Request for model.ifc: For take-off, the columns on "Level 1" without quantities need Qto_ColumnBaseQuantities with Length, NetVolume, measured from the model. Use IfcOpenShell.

First a look at what the model holds.

```python
import ifcopenshell
import ifcopenshell.util.element
import ifcopenshell.util.unit

model = ifcopenshell.open("model.ifc")
print(model.schema)
for unit_type in ("LENGTHUNIT", "AREAUNIT", "VOLUMEUNIT"):
    print(unit_type, ifcopenshell.util.unit.calculate_unit_scale(model, unit_type))
storey = next(s for s in model.by_type("IfcBuildingStorey") if s.Name == "Level 1")
columns = [e for e in ifcopenshell.util.element.get_decomposition(storey) if e.is_a("IfcColumn")]
for e in sorted(columns, key=lambda e: e.id()):
    print(e.id(), e.is_a(), e.Name, list(ifcopenshell.util.element.get_psets(e, qtos_only=True)), sep=" | ")
```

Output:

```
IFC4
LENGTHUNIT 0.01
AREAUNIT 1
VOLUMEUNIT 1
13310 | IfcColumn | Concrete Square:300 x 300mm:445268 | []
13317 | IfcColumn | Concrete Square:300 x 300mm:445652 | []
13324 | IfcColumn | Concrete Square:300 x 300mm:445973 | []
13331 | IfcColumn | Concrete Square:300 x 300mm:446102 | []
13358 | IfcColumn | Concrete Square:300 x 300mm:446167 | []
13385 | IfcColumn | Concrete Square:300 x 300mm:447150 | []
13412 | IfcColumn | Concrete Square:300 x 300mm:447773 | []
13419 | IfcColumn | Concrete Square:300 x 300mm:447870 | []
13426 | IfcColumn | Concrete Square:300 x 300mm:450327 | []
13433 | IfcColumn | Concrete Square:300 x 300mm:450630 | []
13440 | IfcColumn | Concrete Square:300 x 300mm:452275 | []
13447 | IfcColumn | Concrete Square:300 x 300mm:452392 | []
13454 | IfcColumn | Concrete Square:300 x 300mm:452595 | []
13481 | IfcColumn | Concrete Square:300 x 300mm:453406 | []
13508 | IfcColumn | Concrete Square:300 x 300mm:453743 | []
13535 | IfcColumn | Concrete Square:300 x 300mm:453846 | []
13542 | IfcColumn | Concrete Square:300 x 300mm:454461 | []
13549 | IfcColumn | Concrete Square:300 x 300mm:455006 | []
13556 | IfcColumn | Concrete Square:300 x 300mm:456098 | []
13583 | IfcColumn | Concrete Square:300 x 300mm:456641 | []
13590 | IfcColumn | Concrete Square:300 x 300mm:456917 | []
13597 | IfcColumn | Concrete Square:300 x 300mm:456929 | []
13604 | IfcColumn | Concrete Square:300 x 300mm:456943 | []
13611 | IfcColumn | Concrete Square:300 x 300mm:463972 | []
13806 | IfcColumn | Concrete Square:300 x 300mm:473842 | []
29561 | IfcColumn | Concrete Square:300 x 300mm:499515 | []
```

```python
import ifcopenshell
import ifcopenshell.api.pset
import ifcopenshell.geom
import ifcopenshell.util.element
import ifcopenshell.util.shape
import ifcopenshell.util.unit

model = ifcopenshell.open("model.ifc")
unit_scale = ifcopenshell.util.unit.calculate_unit_scale(model)
volume_scale = ifcopenshell.util.unit.calculate_unit_scale(model, "VOLUMEUNIT")
settings = ifcopenshell.geom.settings()

storey = next(s for s in model.by_type("IfcBuildingStorey") if s.Name == "Level 1")
columns = [e for e in ifcopenshell.util.element.get_decomposition(storey) if e.is_a("IfcColumn")]

for e in sorted(columns, key=lambda e: e.id()):
    if ifcopenshell.util.element.get_psets(e, qtos_only=True, should_inherit=False):
        continue
    # Geometry comes back in metres, in the element's own axes.
    shape = ifcopenshell.geom.create_shape(settings, e)
    values = {
        "Length": ifcopenshell.util.shape.get_z(shape.geometry) / unit_scale,
        "NetVolume": ifcopenshell.util.shape.get_volume(shape.geometry) / volume_scale,
    }
    qto = ifcopenshell.api.pset.add_qto(model, product=e, name="Qto_ColumnBaseQuantities")
    ifcopenshell.api.pset.edit_qto(model, qto=qto, properties=values)
    print(e.id(), {k: round(v, 3) for k, v in values.items()})

model.write("model_v2.ifc")
```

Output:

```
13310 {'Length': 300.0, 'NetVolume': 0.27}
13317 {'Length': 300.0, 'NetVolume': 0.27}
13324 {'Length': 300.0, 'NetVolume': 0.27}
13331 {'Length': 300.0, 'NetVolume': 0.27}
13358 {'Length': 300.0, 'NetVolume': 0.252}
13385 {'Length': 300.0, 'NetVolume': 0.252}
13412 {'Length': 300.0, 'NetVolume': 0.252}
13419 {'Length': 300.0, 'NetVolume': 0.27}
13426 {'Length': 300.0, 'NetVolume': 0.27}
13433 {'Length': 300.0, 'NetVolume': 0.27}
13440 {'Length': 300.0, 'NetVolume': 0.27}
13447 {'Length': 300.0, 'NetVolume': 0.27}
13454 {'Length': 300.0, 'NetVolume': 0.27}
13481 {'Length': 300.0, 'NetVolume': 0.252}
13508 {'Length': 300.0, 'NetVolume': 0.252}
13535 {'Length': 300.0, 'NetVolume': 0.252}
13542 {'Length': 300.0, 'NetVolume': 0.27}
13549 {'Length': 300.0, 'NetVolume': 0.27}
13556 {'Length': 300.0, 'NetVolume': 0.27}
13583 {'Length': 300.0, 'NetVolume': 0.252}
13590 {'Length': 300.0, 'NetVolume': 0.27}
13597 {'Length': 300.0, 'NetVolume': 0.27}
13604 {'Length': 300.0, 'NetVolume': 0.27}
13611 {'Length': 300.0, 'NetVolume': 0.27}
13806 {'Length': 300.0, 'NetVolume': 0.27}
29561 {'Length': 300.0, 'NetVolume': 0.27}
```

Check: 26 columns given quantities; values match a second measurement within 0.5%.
